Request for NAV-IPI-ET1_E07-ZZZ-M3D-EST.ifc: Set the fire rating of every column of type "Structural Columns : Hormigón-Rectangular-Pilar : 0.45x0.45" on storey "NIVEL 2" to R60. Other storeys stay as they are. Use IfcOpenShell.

First a look at what the model holds.

```python
import ifcopenshell
import ifcopenshell.util.element

model = ifcopenshell.open("NAV-IPI-ET1_E07-ZZZ-M3D-EST.ifc")
print(model.schema)
storey = next(s for s in model.by_type("IfcBuildingStorey") if s.Name == "NIVEL 2")
columns = [e for e in ifcopenshell.util.element.get_decomposition(storey) if e.is_a("IfcColumn")]
seen = {}
for e in columns:
    element_type = ifcopenshell.util.element.get_type(e)
    key = (element_type.Name if element_type != e and element_type else None, ifcopenshell.util.element.get_pset(e, "Pset_ColumnCommon", "FireRating"))
    seen[key] = seen.get(key, 0) + 1
for (name, value), count in sorted(seen.items(), key=str):
    print(count, "x", name, "|", value)
```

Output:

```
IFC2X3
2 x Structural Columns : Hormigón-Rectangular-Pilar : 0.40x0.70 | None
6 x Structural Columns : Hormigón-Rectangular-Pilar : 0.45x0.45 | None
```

```python
import ifcopenshell
import ifcopenshell.api.pset
import ifcopenshell.util.element

model = ifcopenshell.open("NAV-IPI-ET1_E07-ZZZ-M3D-EST.ifc")

storey = next(s for s in model.by_type("IfcBuildingStorey") if s.Name == "NIVEL 2")
columns = [e for e in ifcopenshell.util.element.get_decomposition(storey) if e.is_a("IfcColumn")]

count = 0
for e in columns:
    element_type = ifcopenshell.util.element.get_type(e)
    if element_type in (None, e) or element_type.Name != "Structural Columns : Hormigón-Rectangular-Pilar : 0.45x0.45":
        continue
    # add_pset returns the element's existing set when there is one.
    pset = ifcopenshell.api.pset.add_pset(model, product=e, name="Pset_ColumnCommon")
    ifcopenshell.api.pset.edit_pset(model, pset=pset, properties={"FireRating": "R60"})
    count += 1

print(count, "columns updated")

model.write("NAV-IPI-ET1_E07-ZZZ-M3D-EST_rev.ifc")
```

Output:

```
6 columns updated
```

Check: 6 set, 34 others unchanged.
